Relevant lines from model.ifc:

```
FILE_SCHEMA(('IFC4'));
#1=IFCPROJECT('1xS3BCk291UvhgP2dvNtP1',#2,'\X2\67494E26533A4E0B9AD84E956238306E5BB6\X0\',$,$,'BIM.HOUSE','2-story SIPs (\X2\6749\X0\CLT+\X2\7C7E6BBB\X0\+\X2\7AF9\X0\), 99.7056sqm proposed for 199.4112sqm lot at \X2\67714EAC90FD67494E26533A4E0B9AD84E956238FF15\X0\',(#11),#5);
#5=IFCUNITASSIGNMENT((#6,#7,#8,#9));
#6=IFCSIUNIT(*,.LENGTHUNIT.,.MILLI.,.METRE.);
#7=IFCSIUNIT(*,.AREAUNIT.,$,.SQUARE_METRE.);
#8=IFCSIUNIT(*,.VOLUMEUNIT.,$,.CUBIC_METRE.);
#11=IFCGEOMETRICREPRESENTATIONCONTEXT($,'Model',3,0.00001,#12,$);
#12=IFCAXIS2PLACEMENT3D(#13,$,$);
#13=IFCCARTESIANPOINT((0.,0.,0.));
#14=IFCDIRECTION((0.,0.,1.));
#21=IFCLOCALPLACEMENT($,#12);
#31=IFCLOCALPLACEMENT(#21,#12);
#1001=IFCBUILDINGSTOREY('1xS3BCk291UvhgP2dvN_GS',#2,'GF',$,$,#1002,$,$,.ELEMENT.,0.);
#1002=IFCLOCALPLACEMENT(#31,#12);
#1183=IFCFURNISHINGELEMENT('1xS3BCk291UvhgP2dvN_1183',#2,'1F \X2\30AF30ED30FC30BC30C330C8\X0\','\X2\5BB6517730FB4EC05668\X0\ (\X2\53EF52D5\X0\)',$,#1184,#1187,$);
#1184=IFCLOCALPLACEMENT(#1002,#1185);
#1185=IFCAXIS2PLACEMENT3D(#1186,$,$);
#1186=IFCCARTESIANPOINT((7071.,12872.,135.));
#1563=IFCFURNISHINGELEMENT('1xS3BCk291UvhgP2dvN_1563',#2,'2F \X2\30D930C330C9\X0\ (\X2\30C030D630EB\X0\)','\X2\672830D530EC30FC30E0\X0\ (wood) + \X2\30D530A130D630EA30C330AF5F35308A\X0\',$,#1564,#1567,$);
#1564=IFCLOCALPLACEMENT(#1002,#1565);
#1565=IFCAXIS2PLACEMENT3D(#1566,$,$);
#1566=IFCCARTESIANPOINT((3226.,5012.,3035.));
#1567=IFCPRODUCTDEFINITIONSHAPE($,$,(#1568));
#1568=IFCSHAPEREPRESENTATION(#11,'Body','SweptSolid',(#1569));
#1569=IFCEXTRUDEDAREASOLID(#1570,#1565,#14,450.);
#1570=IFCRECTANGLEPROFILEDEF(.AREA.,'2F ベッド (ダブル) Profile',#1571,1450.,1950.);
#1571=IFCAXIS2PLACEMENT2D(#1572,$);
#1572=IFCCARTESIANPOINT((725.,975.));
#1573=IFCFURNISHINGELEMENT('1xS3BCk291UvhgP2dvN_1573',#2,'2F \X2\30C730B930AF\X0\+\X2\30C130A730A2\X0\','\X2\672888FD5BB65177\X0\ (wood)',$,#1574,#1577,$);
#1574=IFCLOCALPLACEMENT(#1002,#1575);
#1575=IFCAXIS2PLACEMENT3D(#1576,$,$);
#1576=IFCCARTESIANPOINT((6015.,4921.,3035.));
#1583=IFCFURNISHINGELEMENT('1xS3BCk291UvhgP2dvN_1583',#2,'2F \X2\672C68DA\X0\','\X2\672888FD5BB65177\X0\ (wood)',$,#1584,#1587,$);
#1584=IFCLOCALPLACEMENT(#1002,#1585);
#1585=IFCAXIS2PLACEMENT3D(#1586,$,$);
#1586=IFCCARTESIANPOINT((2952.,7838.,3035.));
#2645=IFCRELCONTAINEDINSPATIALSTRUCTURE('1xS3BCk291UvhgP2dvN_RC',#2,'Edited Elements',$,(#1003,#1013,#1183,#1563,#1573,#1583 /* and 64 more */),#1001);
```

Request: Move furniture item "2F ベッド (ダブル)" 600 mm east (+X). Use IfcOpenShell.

```python
import ifcopenshell
import ifcopenshell.api.geometry
import ifcopenshell.util.placement

model = ifcopenshell.open("model.ifc")

item = model.by_guid("1xS3BCk291UvhgP2dvN_1563")
matrix = ifcopenshell.util.placement.get_local_placement(item.ObjectPlacement)
matrix[0, 3] += 600.0
ifcopenshell.api.geometry.edit_object_placement(model, product=item, matrix=matrix, is_si=False)

print(ifcopenshell.util.placement.get_local_placement(item.ObjectPlacement).round(3) + 0.0)

model.write("model_edited.ifc")
```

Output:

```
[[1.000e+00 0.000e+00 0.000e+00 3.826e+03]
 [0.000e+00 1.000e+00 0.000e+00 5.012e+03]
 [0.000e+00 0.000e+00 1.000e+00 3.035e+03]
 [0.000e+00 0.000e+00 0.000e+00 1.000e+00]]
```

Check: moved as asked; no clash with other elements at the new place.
